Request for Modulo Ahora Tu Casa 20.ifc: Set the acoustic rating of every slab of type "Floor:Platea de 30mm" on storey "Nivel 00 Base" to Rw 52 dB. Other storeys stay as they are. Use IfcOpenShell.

First a look at what the model holds.

```python
import ifcopenshell
import ifcopenshell.util.element

model = ifcopenshell.open("Modulo Ahora Tu Casa 20.ifc")
print(model.schema)
storey = next(s for s in model.by_type("IfcBuildingStorey") if s.Name == "Nivel 00 Base")
slabs = [e for e in ifcopenshell.util.element.get_decomposition(storey) if e.is_a("IfcSlab")]
seen = {}
for e in slabs:
    element_type = ifcopenshell.util.element.get_type(e)
    key = (element_type.Name if element_type != e and element_type else None, ifcopenshell.util.element.get_pset(e, "Pset_SlabCommon", "AcousticRating"))
    seen[key] = seen.get(key, 0) + 1
for (name, value), count in sorted(seen.items(), key=str):
    print(count, "x", name, "|", value)
```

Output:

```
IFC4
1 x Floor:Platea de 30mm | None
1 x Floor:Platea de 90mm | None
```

```python
import ifcopenshell
import ifcopenshell.api.pset
import ifcopenshell.util.element

model = ifcopenshell.open("Modulo Ahora Tu Casa 20.ifc")

storey = next(s for s in model.by_type("IfcBuildingStorey") if s.Name == "Nivel 00 Base")
slabs = [e for e in ifcopenshell.util.element.get_decomposition(storey) if e.is_a("IfcSlab")]

count = 0
for e in slabs:
    element_type = ifcopenshell.util.element.get_type(e)
    if element_type in (None, e) or element_type.Name != "Floor:Platea de 30mm":
        continue
    # add_pset returns the element's existing set when there is one.
    pset = ifcopenshell.api.pset.add_pset(model, product=e, name="Pset_SlabCommon")
    ifcopenshell.api.pset.edit_pset(model, pset=pset, properties={"AcousticRating": "Rw 52 dB"})
    count += 1

print(count, "slabs updated")

model.write("Modulo Ahora Tu Casa 20_updated.ifc")
```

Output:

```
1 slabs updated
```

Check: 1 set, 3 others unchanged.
